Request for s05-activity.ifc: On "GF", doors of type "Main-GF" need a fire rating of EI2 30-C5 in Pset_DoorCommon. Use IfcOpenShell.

First a look at what the model holds.

```python
import ifcopenshell
import ifcopenshell.util.element

model = ifcopenshell.open("s05-activity.ifc")
print(model.schema)
storey = next(s for s in model.by_type("IfcBuildingStorey") if s.Name == "GF")
doors = [e for e in ifcopenshell.util.element.get_decomposition(storey) if e.is_a("IfcDoor")]
seen = {}
for e in doors:
    element_type = ifcopenshell.util.element.get_type(e)
    key = (element_type.Name if element_type != e and element_type else None, ifcopenshell.util.element.get_pset(e, "Pset_DoorCommon", "FireRating"))
    seen[key] = seen.get(key, 0) + 1
for (name, value), count in sorted(seen.items(), key=str):
    print(count, "x", name, "|", value)
```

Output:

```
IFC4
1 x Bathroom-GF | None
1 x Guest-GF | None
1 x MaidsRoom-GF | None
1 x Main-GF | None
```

```python
import ifcopenshell
import ifcopenshell.api.pset
import ifcopenshell.util.element

model = ifcopenshell.open("s05-activity.ifc")

storey = next(s for s in model.by_type("IfcBuildingStorey") if s.Name == "GF")
doors = [e for e in ifcopenshell.util.element.get_decomposition(storey) if e.is_a("IfcDoor")]

count = 0
for e in doors:
    element_type = ifcopenshell.util.element.get_type(e)
    if element_type in (None, e) or element_type.Name != "Main-GF":
        continue
    # add_pset returns the element's existing set when there is one.
    pset = ifcopenshell.api.pset.add_pset(model, product=e, name="Pset_DoorCommon")
    ifcopenshell.api.pset.edit_pset(model, pset=pset, properties={"FireRating": "EI2 30-C5"})
    count += 1

print(count, "doors updated")

model.write("s05-activity_rev.ifc")
```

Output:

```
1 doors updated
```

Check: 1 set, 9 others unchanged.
